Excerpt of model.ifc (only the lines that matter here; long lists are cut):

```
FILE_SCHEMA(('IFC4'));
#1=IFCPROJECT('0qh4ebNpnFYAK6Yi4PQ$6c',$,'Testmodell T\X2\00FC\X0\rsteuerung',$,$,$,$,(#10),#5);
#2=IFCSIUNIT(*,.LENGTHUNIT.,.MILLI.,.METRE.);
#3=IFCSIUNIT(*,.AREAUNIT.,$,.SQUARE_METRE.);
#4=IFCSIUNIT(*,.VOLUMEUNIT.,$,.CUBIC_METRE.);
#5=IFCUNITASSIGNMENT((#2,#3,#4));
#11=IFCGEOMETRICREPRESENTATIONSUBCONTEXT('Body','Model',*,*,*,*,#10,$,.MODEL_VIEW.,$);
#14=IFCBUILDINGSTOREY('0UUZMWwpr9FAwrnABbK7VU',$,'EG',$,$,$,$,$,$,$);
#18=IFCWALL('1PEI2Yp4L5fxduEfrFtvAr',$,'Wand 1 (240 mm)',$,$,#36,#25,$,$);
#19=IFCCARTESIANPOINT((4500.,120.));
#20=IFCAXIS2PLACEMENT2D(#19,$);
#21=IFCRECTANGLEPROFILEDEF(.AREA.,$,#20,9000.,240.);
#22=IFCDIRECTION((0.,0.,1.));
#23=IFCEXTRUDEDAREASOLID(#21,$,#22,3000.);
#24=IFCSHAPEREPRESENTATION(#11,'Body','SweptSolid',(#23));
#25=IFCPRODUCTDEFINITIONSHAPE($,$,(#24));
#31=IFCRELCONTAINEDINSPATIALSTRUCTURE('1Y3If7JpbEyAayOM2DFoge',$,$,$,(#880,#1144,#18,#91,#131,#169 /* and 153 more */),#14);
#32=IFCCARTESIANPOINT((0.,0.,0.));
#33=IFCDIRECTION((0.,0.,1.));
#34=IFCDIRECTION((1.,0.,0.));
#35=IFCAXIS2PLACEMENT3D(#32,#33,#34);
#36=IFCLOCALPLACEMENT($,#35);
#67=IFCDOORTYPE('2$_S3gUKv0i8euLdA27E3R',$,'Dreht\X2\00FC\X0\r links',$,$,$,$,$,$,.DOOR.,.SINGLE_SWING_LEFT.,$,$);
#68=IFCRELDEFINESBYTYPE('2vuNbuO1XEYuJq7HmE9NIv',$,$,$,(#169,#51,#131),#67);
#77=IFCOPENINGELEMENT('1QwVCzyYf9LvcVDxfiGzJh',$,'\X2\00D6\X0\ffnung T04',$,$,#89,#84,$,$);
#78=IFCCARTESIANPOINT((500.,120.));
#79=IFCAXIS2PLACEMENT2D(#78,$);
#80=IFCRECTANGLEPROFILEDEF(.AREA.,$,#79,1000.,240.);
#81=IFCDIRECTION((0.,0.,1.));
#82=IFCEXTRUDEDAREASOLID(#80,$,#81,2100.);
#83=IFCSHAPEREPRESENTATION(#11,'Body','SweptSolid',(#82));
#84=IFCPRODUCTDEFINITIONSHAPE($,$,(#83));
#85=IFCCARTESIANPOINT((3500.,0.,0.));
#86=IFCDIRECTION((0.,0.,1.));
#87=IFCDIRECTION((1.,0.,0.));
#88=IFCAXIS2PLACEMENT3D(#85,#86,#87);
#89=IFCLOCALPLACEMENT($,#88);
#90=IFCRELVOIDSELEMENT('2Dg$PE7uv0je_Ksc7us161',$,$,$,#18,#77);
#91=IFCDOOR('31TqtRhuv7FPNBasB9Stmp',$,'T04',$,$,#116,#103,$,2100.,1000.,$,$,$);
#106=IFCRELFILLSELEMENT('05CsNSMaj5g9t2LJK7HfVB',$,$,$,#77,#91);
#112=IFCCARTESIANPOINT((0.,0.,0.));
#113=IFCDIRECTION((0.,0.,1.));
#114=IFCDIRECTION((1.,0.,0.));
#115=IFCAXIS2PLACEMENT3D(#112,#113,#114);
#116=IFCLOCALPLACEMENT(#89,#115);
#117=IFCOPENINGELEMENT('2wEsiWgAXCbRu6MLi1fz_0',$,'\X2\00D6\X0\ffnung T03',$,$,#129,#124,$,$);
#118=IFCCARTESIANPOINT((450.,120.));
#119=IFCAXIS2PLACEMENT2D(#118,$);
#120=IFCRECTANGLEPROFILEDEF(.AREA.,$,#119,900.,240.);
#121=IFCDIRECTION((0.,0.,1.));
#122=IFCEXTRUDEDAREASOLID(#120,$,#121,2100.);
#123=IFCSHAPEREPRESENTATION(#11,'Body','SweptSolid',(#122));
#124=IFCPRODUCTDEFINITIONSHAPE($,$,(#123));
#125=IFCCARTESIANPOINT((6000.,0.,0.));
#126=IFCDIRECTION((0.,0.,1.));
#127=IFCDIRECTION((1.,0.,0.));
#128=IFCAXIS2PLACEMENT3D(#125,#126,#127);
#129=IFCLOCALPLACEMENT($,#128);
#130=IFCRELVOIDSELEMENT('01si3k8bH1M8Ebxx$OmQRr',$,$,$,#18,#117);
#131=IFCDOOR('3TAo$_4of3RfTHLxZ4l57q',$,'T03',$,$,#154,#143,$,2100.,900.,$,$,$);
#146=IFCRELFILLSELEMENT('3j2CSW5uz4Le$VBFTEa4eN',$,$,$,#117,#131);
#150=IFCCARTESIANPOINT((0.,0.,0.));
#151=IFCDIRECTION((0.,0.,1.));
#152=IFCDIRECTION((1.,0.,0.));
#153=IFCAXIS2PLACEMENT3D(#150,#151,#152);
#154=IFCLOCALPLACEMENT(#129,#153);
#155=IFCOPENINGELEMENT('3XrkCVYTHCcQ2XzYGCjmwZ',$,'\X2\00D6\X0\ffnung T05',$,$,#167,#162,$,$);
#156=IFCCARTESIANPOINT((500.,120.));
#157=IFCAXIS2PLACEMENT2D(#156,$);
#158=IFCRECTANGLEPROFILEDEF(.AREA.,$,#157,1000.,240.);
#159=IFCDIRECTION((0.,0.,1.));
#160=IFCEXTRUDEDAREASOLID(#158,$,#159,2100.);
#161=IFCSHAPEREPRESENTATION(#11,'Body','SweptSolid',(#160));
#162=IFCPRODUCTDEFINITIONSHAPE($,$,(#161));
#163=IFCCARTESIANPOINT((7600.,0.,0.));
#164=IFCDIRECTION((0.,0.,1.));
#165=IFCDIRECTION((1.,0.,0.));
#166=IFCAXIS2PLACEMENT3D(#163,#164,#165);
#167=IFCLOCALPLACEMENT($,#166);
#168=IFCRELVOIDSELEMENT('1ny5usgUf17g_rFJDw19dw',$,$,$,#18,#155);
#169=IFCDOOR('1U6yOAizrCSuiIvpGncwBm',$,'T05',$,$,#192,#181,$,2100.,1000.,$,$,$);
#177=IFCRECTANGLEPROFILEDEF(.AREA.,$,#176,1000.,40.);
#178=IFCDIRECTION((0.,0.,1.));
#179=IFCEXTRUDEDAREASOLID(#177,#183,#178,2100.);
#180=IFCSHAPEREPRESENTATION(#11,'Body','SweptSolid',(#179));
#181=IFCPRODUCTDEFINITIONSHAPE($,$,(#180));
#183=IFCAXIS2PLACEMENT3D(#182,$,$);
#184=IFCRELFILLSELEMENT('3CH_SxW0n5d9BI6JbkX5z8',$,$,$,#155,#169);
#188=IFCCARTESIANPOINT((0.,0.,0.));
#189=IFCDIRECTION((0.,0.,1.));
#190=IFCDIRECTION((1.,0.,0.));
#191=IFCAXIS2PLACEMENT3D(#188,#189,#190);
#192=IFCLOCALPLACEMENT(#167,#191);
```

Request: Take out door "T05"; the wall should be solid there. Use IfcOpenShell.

```python
import ifcopenshell
import ifcopenshell.api.feature
import ifcopenshell.api.root
import ifcopenshell.geom
import ifcopenshell.util.shape

model = ifcopenshell.open("model.ifc")
settings = ifcopenshell.geom.settings()


def volume(element):
    """Net volume in cubic metres, openings subtracted."""
    shape = ifcopenshell.geom.create_shape(settings, element)
    return ifcopenshell.util.shape.get_volume(shape.geometry)


door = model.by_guid("1U6yOAizrCSuiIvpGncwBm")
opening = door.FillsVoids[0].RelatingOpeningElement
wall = opening.VoidsElements[0].RelatingBuildingElement
before = volume(wall)

ifcopenshell.api.root.remove_product(model, product=door)
ifcopenshell.api.feature.remove_feature(model, feature=opening)

after = volume(wall)

print(f"wall volume {before:.3f} -> {after:.3f} m3")

model.write("model_v2.ifc")
```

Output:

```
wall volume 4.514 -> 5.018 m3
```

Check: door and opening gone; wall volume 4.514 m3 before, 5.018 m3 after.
